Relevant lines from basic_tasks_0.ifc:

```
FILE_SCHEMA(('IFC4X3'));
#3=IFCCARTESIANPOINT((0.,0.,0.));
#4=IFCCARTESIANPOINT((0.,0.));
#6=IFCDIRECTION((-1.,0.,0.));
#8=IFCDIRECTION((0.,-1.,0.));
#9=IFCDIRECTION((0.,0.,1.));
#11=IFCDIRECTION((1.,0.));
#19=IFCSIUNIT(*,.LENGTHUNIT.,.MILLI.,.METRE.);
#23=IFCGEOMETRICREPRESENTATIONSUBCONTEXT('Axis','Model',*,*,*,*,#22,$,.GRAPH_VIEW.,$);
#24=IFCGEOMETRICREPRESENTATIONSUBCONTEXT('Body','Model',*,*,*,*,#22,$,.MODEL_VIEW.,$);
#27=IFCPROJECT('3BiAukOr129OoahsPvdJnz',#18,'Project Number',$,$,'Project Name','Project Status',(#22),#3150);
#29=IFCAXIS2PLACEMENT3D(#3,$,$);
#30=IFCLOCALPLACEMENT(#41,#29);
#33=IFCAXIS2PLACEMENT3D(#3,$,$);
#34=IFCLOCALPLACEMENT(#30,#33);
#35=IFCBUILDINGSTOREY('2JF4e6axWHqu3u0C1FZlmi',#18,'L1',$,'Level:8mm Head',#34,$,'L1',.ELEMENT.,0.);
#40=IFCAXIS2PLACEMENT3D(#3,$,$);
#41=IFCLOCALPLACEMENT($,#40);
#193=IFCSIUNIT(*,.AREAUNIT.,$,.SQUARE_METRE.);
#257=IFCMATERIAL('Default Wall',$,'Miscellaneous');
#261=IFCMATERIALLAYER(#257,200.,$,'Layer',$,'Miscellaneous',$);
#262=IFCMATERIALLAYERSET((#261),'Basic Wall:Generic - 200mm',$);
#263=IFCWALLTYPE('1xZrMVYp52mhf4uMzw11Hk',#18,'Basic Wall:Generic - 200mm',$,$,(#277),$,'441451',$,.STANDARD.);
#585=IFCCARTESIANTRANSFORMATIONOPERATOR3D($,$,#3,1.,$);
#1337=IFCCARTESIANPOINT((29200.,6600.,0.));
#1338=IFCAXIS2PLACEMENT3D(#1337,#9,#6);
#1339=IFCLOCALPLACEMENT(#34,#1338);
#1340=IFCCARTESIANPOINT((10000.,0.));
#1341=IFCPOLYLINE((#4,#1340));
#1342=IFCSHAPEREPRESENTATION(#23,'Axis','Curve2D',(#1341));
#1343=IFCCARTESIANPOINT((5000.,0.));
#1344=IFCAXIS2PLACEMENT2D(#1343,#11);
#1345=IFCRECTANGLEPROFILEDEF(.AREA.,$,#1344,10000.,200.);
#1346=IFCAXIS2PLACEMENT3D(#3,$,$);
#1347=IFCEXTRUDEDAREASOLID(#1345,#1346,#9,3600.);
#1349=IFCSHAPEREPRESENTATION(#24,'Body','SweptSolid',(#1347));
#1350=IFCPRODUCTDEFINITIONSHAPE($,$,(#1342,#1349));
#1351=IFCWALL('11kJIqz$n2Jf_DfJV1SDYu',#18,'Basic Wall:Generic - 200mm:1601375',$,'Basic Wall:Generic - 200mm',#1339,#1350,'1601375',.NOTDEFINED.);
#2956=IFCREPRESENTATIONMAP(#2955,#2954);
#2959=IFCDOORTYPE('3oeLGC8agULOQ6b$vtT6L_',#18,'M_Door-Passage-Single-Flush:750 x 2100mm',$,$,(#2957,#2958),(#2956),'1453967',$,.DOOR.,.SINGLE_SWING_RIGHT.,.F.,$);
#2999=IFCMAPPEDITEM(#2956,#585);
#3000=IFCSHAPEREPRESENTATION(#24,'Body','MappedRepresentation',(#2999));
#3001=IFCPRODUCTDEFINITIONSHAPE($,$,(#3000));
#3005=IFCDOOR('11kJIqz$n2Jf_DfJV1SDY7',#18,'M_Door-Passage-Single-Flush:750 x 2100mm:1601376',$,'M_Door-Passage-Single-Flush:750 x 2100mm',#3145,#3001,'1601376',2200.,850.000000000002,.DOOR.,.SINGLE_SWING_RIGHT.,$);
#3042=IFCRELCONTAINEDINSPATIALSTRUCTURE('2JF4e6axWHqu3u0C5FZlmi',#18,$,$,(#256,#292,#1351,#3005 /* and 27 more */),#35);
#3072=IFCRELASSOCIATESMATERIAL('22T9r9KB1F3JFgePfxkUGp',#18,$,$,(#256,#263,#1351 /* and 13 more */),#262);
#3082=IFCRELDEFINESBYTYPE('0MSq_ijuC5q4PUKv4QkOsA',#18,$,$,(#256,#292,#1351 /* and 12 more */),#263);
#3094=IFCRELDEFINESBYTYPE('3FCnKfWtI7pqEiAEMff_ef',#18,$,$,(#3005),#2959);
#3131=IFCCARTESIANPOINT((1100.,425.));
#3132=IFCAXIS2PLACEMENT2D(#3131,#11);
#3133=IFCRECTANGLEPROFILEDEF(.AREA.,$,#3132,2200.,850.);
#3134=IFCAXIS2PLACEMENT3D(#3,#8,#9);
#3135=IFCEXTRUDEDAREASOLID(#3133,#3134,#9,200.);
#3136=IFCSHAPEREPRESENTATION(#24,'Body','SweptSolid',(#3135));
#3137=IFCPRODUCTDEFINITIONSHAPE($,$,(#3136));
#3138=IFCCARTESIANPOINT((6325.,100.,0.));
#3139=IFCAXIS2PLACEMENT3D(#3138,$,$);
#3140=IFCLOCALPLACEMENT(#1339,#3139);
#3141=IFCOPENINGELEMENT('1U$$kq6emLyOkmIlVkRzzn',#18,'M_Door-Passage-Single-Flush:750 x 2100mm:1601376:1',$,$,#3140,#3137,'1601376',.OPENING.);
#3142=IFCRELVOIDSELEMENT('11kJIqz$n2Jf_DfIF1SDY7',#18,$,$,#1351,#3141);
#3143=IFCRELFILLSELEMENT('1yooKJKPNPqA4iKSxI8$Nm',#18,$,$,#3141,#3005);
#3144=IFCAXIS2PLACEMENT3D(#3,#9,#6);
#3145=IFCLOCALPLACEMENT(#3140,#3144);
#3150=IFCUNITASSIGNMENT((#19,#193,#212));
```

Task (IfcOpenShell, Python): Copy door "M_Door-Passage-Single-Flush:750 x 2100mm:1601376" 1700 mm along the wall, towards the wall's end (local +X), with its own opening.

```python
import ifcopenshell
import ifcopenshell.api.feature
import ifcopenshell.api.geometry
import ifcopenshell.api.root
import ifcopenshell.geom
import ifcopenshell.util.element
import ifcopenshell.util.placement
import ifcopenshell.util.shape

model = ifcopenshell.open("basic_tasks_0.ifc")
settings = ifcopenshell.geom.settings()


def volume(element):
    """Net volume in cubic metres, openings subtracted."""
    shape = ifcopenshell.geom.create_shape(settings, element)
    return ifcopenshell.util.shape.get_volume(shape.geometry)


def reuse_history(source, copy):
    """copy_class also copies each property set's owner history, people and application; keep the originals."""
    for rel in copy.IsDefinedBy:
        if rel.is_a("IfcRelDefinesByProperties") and (history := rel.RelatingPropertyDefinition.OwnerHistory):
            rel.RelatingPropertyDefinition.OwnerHistory = source.OwnerHistory
            ifcopenshell.util.element.remove_deep2(model, history)


door = model.by_id(3005)
opening = door.FillsVoids[0].RelatingOpeningElement
wall = opening.VoidsElements[0].RelatingBuildingElement
before = volume(wall)
shift = ifcopenshell.util.placement.get_local_placement(wall.ObjectPlacement)[:3, 0] * 1700.0

# copy_class copies the void relationship, type, container and properties, but no geometry.
new_opening = ifcopenshell.api.root.copy_class(model, product=opening)
new_opening.Representation = ifcopenshell.util.element.copy_deep(
    model, opening.Representation, exclude=["IfcGeometricRepresentationContext", "IfcRepresentationMap"]
)
new_opening.Name = "M_Door-Passage-Single-Flush:750 x 2100mm"
new_opening.Tag = None
new_door = ifcopenshell.api.root.copy_class(model, product=door)
new_door.Representation = ifcopenshell.util.element.copy_deep(
    model, door.Representation, exclude=["IfcGeometricRepresentationContext", "IfcRepresentationMap"]
)
new_door.Name = "M_Door-Passage-Single-Flush:750 x 2100mm"
new_door.Tag = None
reuse_history(door, new_door)
ifcopenshell.api.feature.add_filling(model, opening=new_opening, element=new_door)

for old, new in ((opening, new_opening), (door, new_door)):
    matrix = ifcopenshell.util.placement.get_local_placement(old.ObjectPlacement)
    matrix[:3, 3] += shift
    ifcopenshell.api.geometry.edit_object_placement(model, product=new, matrix=matrix, is_si=False)

after = volume(wall)

print(f"wall volume {before:.3f} -> {after:.3f} m3")

model.write("basic_tasks_0-out.ifc")
```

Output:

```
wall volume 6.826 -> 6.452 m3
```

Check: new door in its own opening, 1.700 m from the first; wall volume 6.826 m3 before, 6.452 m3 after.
